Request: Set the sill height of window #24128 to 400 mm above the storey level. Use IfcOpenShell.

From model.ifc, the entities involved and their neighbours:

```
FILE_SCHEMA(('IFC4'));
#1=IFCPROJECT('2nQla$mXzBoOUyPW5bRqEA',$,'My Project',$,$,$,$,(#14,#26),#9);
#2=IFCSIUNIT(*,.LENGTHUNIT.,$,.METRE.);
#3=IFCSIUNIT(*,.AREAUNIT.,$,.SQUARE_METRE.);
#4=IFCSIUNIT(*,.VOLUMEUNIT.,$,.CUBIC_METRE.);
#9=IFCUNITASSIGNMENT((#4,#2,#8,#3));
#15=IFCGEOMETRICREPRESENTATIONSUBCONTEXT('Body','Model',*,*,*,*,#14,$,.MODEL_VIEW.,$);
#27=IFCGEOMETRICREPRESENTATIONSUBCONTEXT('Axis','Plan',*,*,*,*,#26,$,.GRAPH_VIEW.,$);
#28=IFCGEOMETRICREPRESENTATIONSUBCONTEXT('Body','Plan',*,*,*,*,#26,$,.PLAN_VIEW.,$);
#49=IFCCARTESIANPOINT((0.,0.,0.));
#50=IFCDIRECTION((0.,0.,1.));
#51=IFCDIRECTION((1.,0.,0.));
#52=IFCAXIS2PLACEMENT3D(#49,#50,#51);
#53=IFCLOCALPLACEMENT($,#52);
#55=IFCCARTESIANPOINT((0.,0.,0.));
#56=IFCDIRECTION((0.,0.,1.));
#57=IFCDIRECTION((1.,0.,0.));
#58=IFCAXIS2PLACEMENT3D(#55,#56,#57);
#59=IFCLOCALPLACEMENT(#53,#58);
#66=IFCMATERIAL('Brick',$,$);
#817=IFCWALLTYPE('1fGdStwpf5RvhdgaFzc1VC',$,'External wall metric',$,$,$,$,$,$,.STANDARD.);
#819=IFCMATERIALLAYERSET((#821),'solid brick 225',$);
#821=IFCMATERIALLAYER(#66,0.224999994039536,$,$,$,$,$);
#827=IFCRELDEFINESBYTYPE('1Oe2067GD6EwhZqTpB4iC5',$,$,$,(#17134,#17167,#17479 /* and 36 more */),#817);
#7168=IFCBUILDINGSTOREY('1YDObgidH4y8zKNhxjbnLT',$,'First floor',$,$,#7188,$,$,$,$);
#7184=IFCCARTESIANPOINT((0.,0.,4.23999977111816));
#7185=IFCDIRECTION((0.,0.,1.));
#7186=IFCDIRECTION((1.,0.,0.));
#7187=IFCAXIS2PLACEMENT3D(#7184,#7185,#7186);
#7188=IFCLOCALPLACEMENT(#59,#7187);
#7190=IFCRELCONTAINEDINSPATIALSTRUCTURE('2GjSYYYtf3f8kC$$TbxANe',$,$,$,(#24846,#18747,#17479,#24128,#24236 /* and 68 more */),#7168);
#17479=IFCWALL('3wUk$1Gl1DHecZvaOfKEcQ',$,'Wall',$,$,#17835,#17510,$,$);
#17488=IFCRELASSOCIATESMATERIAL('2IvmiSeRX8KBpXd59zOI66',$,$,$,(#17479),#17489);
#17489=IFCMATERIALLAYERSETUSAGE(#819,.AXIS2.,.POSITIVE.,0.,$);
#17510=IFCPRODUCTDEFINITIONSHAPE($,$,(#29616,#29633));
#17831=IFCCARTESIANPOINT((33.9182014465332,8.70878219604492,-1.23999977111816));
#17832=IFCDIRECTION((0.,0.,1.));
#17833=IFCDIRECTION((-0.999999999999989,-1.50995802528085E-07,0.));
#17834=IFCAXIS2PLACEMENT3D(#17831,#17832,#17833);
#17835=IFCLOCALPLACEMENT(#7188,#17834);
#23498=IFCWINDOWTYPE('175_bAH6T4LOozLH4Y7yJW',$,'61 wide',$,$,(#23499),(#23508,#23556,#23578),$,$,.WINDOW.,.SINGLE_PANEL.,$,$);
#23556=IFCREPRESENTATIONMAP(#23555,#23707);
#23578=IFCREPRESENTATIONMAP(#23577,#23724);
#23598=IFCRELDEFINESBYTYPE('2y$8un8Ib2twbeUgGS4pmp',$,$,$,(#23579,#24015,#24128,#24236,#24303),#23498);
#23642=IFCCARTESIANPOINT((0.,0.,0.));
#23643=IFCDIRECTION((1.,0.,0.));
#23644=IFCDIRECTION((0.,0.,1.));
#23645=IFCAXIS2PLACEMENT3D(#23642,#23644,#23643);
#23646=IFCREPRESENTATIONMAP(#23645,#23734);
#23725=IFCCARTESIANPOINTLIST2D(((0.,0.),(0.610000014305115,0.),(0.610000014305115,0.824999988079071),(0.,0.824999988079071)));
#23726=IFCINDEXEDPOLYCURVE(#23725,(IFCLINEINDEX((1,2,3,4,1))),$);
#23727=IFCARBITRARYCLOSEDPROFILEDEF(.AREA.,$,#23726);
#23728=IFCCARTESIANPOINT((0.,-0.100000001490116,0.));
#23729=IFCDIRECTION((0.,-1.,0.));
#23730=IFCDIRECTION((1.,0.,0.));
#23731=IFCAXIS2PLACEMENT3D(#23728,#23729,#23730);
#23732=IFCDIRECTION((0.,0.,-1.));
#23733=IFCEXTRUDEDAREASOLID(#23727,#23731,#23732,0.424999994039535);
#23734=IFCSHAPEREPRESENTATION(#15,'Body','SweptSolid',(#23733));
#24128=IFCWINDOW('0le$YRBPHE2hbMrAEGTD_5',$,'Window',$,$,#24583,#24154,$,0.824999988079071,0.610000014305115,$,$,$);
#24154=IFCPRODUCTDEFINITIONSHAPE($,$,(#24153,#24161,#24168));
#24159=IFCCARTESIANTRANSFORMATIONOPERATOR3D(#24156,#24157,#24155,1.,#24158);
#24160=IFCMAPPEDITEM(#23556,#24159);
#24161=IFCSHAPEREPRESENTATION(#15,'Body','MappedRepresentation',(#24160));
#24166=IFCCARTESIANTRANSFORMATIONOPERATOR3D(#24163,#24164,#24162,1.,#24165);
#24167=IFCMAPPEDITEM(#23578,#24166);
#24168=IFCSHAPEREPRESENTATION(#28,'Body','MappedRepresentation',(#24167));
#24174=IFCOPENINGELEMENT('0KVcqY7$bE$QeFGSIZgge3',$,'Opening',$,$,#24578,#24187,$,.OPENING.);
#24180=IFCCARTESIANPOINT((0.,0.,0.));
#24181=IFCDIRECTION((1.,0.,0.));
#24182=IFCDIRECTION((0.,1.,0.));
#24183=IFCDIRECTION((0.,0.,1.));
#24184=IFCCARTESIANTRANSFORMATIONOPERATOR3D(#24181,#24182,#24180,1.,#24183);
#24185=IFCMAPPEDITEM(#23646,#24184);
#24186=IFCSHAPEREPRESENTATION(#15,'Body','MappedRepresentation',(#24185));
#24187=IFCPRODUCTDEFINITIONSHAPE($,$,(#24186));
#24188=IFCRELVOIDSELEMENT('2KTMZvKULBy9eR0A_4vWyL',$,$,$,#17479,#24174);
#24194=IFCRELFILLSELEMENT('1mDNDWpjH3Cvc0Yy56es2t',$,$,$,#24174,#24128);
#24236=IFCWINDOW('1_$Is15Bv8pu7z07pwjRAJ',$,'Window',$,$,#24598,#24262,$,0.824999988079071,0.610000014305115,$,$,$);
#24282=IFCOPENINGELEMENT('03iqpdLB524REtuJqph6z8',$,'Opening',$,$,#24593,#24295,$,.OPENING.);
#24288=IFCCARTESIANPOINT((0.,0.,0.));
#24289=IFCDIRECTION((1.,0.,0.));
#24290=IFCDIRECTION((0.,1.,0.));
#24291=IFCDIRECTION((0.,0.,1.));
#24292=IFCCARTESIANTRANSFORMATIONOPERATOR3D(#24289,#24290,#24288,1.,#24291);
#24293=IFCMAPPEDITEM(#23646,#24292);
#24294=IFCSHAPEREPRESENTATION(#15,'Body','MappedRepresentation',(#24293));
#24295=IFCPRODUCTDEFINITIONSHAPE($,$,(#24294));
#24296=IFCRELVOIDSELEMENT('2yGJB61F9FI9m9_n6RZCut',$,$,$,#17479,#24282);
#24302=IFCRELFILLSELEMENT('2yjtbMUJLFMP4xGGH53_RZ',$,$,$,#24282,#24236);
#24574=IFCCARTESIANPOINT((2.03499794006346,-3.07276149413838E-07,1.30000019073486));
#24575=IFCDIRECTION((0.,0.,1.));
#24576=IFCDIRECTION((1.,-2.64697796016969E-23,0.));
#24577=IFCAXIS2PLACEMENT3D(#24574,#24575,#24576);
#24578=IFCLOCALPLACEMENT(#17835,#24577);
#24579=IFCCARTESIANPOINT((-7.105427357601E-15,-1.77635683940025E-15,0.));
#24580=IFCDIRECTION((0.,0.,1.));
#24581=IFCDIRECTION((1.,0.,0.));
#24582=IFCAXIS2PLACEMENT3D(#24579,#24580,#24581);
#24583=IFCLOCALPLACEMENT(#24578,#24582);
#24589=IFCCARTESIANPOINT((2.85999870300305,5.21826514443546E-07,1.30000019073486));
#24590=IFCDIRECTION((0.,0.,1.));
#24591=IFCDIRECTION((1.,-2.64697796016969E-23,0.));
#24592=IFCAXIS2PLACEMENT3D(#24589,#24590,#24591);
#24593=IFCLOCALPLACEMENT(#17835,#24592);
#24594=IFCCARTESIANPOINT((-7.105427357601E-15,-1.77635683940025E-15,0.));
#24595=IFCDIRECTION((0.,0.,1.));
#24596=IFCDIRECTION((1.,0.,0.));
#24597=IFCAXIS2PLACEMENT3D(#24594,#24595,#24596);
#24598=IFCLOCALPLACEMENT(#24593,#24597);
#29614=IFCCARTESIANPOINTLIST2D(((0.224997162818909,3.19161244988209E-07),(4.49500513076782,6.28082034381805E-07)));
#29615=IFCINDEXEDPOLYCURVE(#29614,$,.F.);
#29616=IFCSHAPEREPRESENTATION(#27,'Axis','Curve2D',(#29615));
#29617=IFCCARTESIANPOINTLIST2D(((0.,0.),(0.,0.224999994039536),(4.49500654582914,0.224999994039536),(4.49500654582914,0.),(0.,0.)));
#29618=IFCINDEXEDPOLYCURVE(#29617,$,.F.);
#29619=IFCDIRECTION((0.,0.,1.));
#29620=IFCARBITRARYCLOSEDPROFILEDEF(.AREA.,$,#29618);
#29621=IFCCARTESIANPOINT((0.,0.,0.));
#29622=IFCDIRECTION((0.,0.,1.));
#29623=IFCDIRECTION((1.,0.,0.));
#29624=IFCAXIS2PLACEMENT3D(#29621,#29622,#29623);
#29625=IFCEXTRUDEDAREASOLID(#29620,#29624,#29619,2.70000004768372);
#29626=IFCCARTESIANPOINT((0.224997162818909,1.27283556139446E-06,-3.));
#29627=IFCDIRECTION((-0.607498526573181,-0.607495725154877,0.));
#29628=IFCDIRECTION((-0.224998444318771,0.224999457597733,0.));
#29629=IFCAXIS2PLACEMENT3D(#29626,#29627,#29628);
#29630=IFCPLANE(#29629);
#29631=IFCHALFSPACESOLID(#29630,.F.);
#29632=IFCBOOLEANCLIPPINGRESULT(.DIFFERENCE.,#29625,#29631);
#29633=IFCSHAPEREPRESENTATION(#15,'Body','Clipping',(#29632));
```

```python
import numpy as np
import ifcopenshell
import ifcopenshell.api.geometry
import ifcopenshell.geom
import ifcopenshell.util.element
import ifcopenshell.util.placement
import ifcopenshell.util.shape
import ifcopenshell.util.unit

model = ifcopenshell.open("model.ifc")
unit_scale = ifcopenshell.util.unit.calculate_unit_scale(model)

window = model.by_guid("0le$YRBPHE2hbMrAEGTD_5")
opening = window.FillsVoids[0].RelatingOpeningElement
storey = ifcopenshell.util.element.get_container(window, ifc_class="IfcBuildingStorey")
level = ifcopenshell.util.placement.get_local_placement(storey.ObjectPlacement)[2, 3]

# The opening's origin need not be at the sill, so measure its lowest point.
shape = ifcopenshell.geom.create_shape(ifcopenshell.geom.settings(), opening)
bottom = ifcopenshell.util.shape.get_shape_bottom_elevation(shape, shape.geometry) / unit_scale
dz = level + 0.4 / unit_scale - bottom

shift = np.array([0.0, 0.0, dz])
# The window is placed relative to its opening, so it follows when the opening moves.
matrix = ifcopenshell.util.placement.get_local_placement(opening.ObjectPlacement)
matrix[:3, 3] += shift
ifcopenshell.api.geometry.edit_object_placement(
    model, product=opening, matrix=matrix, is_si=False, should_transform_children=True
)

print(f"moved by {dz * unit_scale:+.3f} m")

model.write("model_updated.ifc")
```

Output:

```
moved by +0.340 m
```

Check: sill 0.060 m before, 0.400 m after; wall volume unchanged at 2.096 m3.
